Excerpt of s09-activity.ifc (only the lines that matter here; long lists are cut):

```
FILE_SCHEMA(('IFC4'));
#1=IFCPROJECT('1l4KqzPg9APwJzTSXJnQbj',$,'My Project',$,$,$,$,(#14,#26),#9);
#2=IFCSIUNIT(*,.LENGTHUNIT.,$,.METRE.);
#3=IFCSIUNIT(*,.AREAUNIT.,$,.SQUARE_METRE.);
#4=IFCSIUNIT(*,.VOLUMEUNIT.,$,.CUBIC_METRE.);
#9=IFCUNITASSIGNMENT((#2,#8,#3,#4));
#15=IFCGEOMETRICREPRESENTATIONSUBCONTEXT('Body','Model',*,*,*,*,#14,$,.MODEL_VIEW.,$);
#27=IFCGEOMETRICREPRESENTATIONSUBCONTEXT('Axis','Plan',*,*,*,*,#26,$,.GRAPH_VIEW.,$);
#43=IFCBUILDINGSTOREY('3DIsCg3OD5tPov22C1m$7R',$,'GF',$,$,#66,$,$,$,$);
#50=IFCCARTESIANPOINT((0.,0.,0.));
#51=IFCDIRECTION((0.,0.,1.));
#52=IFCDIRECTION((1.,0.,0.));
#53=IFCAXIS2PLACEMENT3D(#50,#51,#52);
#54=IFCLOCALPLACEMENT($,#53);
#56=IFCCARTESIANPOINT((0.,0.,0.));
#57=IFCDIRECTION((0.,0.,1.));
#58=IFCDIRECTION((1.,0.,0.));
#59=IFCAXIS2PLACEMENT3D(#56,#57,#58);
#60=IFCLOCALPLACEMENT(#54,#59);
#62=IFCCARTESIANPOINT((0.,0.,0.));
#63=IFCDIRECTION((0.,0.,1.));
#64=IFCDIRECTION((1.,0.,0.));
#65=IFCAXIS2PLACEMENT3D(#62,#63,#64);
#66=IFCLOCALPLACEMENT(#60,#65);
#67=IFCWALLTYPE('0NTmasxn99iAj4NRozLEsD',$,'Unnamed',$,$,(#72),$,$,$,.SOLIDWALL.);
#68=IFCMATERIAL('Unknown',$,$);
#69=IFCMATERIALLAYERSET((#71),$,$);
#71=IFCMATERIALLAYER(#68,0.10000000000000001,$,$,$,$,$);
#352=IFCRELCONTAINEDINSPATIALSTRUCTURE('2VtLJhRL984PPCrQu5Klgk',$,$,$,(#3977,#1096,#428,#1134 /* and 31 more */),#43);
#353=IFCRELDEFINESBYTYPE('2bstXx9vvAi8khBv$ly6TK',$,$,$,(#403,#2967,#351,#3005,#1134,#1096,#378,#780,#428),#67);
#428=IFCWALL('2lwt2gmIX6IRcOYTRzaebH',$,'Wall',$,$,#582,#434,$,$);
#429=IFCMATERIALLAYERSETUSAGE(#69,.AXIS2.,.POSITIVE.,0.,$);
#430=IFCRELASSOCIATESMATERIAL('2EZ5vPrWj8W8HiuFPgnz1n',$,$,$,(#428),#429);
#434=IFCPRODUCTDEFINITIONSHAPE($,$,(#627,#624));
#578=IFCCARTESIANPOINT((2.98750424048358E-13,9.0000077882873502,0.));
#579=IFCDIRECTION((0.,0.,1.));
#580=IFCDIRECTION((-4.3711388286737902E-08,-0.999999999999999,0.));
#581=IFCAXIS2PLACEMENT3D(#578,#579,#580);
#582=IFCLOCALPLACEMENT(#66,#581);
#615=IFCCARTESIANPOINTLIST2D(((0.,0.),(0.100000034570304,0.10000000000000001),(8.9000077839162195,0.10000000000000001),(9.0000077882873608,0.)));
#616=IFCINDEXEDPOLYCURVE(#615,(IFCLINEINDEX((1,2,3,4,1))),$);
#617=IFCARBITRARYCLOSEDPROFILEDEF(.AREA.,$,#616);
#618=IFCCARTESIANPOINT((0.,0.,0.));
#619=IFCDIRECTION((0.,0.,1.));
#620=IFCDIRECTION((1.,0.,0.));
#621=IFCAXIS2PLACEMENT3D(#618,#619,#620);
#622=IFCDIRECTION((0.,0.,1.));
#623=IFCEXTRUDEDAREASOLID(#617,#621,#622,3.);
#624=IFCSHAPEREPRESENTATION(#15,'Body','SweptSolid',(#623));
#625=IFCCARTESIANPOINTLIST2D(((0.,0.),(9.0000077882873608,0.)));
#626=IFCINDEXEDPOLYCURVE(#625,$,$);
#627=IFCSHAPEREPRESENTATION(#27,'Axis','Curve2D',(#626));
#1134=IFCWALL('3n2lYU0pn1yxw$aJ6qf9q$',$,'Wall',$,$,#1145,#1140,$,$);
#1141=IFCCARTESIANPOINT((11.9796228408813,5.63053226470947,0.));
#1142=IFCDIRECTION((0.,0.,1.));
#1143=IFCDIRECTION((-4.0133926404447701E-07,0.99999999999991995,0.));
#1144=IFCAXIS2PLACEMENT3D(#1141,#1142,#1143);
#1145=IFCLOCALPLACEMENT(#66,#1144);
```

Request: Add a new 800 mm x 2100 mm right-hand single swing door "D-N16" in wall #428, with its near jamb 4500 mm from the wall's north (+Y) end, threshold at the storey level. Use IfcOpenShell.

```python
import numpy as np
import ifcopenshell
import ifcopenshell.api.feature
import ifcopenshell.api.geometry
import ifcopenshell.api.root
import ifcopenshell.api.spatial
import ifcopenshell.geom
import ifcopenshell.util.element
import ifcopenshell.util.placement
import ifcopenshell.util.representation
import ifcopenshell.util.shape
import ifcopenshell.util.unit

model = ifcopenshell.open("s09-activity.ifc")
unit_scale = ifcopenshell.util.unit.calculate_unit_scale(model)
settings = ifcopenshell.geom.settings()


def volume(element):
    """Net volume in cubic metres, openings subtracted."""
    shape = ifcopenshell.geom.create_shape(settings, element)
    return ifcopenshell.util.shape.get_volume(shape.geometry)


wall = model.by_id(428)
storey = ifcopenshell.util.element.get_container(wall, ifc_class="IfcBuildingStorey")
context = ifcopenshell.util.representation.get_context(model, "Model", "Body", "MODEL_VIEW")
before = volume(wall)

width, height, from_end, sill = 0.8, 2.1, 4.5, 0.0  # metres

# The wall runs along its own X axis, and the end named is its -X end.
wall_shape = ifcopenshell.geom.create_shape(settings, wall)
x, y, z = ifcopenshell.util.shape.get_vertices(wall_shape.geometry).T
start = x.min() + from_end
face, thickness = float(y.min()), float(y.max() - y.min())
wall_matrix = ifcopenshell.util.placement.get_local_placement(wall.ObjectPlacement)
level = ifcopenshell.util.placement.get_local_placement(storey.ObjectPlacement)[2, 3]


def in_wall(x, y):
    """Placement at x, y metres in the wall's axes, at sill height."""
    matrix = wall_matrix.copy()
    matrix[:, 3] = wall_matrix @ np.array([x / unit_scale, y / unit_scale, 0.0, 1.0])
    matrix[2, 3] = level + sill / unit_scale
    return matrix


# Opening: a box that overshoots both wall faces by 50 mm.
opening = ifcopenshell.api.root.create_entity(model, ifc_class="IfcOpeningElement", predefined_type="OPENING")
box = ifcopenshell.api.geometry.add_wall_representation(
    model, context=context, length=width, height=height, thickness=thickness + 0.1
)
ifcopenshell.api.geometry.assign_representation(model, product=opening, representation=box)
ifcopenshell.api.geometry.edit_object_placement(model, product=opening, matrix=in_wall(start, face - 0.05), is_si=False)
ifcopenshell.api.feature.add_feature(model, feature=opening, element=wall)

door = ifcopenshell.api.root.create_entity(model, ifc_class="IfcDoor", name="D-N16", predefined_type="DOOR")
door.OverallWidth, door.OverallHeight = width / unit_scale, height / unit_scale
door.OperationType = "SINGLE_SWING_RIGHT"
body = ifcopenshell.api.geometry.add_door_representation(
    model,
    context=context,
    overall_width=door.OverallWidth,
    overall_height=door.OverallHeight,
    operation_type="SINGLE_SWING_RIGHT",
    lining_properties={"LiningDepth": thickness / unit_scale, "ThresholdDepth": thickness / unit_scale},
)
ifcopenshell.api.geometry.assign_representation(model, product=door, representation=body)
ifcopenshell.api.spatial.assign_container(model, products=[door], relating_structure=storey)
ifcopenshell.api.feature.add_filling(model, opening=opening, element=door)

# The lining spans the wall, so the door starts at the wall face.
ifcopenshell.api.geometry.edit_object_placement(model, product=door, matrix=in_wall(start, face), is_si=False)

after = volume(wall)

print(f"wall volume {before:.3f} -> {after:.3f} m3")

model.write("s09-activity_updated.ifc")
```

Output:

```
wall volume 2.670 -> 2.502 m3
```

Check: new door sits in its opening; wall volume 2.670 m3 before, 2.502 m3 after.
